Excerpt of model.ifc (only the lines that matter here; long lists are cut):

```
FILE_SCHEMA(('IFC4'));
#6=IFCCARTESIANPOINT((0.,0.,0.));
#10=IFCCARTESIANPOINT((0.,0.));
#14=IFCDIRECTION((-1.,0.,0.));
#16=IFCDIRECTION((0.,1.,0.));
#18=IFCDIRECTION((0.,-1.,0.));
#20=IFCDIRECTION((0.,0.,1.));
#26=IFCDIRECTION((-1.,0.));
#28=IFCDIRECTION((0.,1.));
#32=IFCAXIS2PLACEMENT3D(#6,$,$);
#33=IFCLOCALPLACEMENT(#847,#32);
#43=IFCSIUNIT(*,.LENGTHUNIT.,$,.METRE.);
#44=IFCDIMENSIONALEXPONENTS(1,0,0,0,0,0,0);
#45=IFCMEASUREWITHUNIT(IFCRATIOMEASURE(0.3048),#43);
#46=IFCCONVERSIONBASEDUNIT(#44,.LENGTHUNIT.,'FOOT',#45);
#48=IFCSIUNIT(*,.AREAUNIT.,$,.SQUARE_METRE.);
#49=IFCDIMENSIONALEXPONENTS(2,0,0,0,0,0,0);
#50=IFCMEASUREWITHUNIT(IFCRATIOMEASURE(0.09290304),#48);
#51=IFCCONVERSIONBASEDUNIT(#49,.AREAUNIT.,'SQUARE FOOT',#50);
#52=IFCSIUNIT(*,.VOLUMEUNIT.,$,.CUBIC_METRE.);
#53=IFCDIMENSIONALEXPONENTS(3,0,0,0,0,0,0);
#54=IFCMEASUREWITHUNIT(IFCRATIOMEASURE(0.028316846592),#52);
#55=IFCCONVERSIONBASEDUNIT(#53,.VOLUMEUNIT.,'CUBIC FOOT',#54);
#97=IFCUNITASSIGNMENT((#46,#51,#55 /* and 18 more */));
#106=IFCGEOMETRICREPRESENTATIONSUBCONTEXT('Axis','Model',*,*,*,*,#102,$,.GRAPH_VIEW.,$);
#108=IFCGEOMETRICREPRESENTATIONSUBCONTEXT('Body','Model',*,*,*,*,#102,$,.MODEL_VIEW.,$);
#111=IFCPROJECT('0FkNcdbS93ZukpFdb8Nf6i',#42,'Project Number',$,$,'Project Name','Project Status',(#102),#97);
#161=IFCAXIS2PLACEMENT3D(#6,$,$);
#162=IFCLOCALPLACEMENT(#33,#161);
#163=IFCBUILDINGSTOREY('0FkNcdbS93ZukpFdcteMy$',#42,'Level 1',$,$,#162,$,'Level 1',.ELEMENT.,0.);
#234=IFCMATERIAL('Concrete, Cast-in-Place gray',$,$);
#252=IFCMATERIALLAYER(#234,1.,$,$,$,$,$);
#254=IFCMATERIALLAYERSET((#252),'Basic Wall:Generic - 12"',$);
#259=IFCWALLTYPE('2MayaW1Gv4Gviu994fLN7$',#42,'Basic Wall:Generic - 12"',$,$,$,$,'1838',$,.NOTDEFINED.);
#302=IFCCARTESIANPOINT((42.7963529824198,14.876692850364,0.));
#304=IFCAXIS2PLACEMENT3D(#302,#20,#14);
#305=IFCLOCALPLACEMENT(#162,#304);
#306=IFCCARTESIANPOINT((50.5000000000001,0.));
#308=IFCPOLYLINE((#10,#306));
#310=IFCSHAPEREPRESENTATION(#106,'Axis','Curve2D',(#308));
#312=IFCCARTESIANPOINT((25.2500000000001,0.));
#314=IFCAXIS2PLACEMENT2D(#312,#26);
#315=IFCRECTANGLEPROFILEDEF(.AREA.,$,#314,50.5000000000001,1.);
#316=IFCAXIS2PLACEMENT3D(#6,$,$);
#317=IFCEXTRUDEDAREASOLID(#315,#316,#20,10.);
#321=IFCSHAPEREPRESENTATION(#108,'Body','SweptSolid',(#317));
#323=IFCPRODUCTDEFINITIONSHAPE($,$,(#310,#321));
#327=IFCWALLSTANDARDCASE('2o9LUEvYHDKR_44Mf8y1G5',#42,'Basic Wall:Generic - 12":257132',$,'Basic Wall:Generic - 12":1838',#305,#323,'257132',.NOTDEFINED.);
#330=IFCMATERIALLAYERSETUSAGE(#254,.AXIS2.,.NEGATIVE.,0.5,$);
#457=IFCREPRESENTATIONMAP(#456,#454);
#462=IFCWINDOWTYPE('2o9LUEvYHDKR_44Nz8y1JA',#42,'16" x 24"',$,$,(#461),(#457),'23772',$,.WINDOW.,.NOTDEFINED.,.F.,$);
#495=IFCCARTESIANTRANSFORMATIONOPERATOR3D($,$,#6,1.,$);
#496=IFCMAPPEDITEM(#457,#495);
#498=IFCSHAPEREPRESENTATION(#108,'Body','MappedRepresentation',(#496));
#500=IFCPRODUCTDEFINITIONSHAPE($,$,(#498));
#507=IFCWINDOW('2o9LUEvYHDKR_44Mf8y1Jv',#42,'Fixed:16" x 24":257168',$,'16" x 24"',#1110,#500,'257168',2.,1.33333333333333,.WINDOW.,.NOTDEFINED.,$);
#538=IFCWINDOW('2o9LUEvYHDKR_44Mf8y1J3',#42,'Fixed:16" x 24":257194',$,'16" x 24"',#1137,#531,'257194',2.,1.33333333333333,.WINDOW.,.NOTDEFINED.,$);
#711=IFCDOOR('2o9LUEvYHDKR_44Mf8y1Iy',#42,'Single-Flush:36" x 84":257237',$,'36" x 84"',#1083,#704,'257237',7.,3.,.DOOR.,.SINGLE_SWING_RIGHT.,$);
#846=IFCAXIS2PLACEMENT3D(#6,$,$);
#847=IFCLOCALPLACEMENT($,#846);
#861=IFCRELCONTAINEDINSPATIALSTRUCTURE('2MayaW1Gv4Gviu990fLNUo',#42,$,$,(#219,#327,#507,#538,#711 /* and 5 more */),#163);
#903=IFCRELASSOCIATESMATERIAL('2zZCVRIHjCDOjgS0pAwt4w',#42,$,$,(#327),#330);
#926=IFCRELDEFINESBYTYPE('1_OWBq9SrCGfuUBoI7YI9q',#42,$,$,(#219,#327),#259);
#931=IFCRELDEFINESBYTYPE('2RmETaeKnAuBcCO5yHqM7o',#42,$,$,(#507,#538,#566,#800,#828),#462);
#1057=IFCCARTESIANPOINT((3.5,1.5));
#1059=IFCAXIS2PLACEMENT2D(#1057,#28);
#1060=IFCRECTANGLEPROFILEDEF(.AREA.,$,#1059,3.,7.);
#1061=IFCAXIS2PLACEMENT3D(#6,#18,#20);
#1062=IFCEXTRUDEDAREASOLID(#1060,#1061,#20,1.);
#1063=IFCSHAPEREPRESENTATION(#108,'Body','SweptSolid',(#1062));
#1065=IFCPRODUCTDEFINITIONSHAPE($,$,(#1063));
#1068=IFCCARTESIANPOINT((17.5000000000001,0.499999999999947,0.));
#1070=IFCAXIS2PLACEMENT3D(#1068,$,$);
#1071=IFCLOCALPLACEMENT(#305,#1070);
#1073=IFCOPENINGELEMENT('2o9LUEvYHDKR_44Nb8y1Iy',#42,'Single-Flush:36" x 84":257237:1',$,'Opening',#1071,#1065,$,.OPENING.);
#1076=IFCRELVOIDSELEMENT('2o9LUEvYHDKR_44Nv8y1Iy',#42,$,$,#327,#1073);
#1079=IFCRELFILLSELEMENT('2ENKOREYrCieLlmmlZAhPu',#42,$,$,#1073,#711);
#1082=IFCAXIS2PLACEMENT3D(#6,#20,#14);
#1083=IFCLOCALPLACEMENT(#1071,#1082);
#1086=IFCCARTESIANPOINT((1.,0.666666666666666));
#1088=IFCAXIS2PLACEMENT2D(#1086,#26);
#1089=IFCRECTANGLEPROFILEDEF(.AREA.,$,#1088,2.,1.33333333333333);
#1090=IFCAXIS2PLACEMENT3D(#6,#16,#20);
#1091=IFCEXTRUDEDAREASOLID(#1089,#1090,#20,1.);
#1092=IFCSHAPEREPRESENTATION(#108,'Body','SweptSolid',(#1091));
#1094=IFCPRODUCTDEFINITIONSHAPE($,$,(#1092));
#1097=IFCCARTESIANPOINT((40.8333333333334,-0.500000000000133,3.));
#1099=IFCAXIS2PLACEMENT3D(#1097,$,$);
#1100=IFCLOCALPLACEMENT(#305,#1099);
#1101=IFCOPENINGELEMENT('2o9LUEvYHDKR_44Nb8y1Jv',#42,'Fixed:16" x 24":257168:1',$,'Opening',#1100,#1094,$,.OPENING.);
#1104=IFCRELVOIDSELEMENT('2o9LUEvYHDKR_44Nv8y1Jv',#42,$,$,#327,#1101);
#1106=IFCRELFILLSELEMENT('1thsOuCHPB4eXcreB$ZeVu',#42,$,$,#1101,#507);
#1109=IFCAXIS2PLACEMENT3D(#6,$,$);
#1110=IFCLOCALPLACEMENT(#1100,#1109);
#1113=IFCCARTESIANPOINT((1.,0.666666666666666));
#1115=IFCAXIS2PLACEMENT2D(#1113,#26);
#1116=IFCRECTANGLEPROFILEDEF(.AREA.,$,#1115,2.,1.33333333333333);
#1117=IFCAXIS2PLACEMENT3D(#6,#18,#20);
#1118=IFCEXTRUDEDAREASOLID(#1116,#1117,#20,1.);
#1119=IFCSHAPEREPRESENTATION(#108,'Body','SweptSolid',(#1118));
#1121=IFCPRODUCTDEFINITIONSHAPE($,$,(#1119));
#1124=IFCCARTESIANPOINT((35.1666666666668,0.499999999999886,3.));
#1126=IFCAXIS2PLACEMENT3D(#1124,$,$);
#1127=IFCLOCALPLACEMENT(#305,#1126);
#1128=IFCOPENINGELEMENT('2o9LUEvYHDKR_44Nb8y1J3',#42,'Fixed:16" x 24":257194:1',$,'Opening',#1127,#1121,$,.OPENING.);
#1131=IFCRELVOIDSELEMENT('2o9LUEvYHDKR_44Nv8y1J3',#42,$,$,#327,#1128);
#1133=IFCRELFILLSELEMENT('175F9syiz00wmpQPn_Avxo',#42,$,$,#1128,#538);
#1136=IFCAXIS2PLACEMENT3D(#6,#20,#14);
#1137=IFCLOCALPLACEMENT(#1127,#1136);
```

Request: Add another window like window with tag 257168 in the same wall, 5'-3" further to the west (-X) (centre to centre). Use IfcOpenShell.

```python
import ifcopenshell
import ifcopenshell.api.feature
import ifcopenshell.api.geometry
import ifcopenshell.api.root
import ifcopenshell.geom
import ifcopenshell.util.element
import ifcopenshell.util.placement
import ifcopenshell.util.shape
import ifcopenshell.util.unit

model = ifcopenshell.open("model.ifc")
unit_scale = ifcopenshell.util.unit.calculate_unit_scale(model)
settings = ifcopenshell.geom.settings()


def volume(element):
    """Net volume in cubic metres, openings subtracted."""
    shape = ifcopenshell.geom.create_shape(settings, element)
    return ifcopenshell.util.shape.get_volume(shape.geometry)


def reuse_history(source, copy):
    """copy_class also copies each property set's owner history, people and application; keep the originals."""
    for rel in copy.IsDefinedBy:
        if rel.is_a("IfcRelDefinesByProperties") and (history := rel.RelatingPropertyDefinition.OwnerHistory):
            rel.RelatingPropertyDefinition.OwnerHistory = source.OwnerHistory
            ifcopenshell.util.element.remove_deep2(model, history)


window = model.by_guid("2o9LUEvYHDKR_44Mf8y1Jv")
opening = window.FillsVoids[0].RelatingOpeningElement
wall = opening.VoidsElements[0].RelatingBuildingElement
before = volume(wall)
shift = ifcopenshell.util.placement.get_local_placement(wall.ObjectPlacement)[:3, 0] * 63 * 0.0254 / unit_scale

# copy_class copies the void relationship, type, container and properties, but no geometry.
new_opening = ifcopenshell.api.root.copy_class(model, product=opening)
new_opening.Representation = ifcopenshell.util.element.copy_deep(
    model, opening.Representation, exclude=["IfcGeometricRepresentationContext", "IfcRepresentationMap"]
)
new_opening.Name = 'Fixed:16" x 24"'
new_window = ifcopenshell.api.root.copy_class(model, product=window)
new_window.Representation = ifcopenshell.util.element.copy_deep(
    model, window.Representation, exclude=["IfcGeometricRepresentationContext", "IfcRepresentationMap"]
)
new_window.Name = 'Fixed:16" x 24"'
new_window.Tag = None
reuse_history(window, new_window)
ifcopenshell.api.feature.add_filling(model, opening=new_opening, element=new_window)

for old, new in ((opening, new_opening), (window, new_window)):
    matrix = ifcopenshell.util.placement.get_local_placement(old.ObjectPlacement)
    matrix[:3, 3] += shift
    ifcopenshell.api.geometry.edit_object_placement(model, product=new, matrix=matrix, is_si=False)

after = volume(wall)

print(f"wall volume {before:.3f} -> {after:.3f} m3")

model.write("model_v2.ifc")
```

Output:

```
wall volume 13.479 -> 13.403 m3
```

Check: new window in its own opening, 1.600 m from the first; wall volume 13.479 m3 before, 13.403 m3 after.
